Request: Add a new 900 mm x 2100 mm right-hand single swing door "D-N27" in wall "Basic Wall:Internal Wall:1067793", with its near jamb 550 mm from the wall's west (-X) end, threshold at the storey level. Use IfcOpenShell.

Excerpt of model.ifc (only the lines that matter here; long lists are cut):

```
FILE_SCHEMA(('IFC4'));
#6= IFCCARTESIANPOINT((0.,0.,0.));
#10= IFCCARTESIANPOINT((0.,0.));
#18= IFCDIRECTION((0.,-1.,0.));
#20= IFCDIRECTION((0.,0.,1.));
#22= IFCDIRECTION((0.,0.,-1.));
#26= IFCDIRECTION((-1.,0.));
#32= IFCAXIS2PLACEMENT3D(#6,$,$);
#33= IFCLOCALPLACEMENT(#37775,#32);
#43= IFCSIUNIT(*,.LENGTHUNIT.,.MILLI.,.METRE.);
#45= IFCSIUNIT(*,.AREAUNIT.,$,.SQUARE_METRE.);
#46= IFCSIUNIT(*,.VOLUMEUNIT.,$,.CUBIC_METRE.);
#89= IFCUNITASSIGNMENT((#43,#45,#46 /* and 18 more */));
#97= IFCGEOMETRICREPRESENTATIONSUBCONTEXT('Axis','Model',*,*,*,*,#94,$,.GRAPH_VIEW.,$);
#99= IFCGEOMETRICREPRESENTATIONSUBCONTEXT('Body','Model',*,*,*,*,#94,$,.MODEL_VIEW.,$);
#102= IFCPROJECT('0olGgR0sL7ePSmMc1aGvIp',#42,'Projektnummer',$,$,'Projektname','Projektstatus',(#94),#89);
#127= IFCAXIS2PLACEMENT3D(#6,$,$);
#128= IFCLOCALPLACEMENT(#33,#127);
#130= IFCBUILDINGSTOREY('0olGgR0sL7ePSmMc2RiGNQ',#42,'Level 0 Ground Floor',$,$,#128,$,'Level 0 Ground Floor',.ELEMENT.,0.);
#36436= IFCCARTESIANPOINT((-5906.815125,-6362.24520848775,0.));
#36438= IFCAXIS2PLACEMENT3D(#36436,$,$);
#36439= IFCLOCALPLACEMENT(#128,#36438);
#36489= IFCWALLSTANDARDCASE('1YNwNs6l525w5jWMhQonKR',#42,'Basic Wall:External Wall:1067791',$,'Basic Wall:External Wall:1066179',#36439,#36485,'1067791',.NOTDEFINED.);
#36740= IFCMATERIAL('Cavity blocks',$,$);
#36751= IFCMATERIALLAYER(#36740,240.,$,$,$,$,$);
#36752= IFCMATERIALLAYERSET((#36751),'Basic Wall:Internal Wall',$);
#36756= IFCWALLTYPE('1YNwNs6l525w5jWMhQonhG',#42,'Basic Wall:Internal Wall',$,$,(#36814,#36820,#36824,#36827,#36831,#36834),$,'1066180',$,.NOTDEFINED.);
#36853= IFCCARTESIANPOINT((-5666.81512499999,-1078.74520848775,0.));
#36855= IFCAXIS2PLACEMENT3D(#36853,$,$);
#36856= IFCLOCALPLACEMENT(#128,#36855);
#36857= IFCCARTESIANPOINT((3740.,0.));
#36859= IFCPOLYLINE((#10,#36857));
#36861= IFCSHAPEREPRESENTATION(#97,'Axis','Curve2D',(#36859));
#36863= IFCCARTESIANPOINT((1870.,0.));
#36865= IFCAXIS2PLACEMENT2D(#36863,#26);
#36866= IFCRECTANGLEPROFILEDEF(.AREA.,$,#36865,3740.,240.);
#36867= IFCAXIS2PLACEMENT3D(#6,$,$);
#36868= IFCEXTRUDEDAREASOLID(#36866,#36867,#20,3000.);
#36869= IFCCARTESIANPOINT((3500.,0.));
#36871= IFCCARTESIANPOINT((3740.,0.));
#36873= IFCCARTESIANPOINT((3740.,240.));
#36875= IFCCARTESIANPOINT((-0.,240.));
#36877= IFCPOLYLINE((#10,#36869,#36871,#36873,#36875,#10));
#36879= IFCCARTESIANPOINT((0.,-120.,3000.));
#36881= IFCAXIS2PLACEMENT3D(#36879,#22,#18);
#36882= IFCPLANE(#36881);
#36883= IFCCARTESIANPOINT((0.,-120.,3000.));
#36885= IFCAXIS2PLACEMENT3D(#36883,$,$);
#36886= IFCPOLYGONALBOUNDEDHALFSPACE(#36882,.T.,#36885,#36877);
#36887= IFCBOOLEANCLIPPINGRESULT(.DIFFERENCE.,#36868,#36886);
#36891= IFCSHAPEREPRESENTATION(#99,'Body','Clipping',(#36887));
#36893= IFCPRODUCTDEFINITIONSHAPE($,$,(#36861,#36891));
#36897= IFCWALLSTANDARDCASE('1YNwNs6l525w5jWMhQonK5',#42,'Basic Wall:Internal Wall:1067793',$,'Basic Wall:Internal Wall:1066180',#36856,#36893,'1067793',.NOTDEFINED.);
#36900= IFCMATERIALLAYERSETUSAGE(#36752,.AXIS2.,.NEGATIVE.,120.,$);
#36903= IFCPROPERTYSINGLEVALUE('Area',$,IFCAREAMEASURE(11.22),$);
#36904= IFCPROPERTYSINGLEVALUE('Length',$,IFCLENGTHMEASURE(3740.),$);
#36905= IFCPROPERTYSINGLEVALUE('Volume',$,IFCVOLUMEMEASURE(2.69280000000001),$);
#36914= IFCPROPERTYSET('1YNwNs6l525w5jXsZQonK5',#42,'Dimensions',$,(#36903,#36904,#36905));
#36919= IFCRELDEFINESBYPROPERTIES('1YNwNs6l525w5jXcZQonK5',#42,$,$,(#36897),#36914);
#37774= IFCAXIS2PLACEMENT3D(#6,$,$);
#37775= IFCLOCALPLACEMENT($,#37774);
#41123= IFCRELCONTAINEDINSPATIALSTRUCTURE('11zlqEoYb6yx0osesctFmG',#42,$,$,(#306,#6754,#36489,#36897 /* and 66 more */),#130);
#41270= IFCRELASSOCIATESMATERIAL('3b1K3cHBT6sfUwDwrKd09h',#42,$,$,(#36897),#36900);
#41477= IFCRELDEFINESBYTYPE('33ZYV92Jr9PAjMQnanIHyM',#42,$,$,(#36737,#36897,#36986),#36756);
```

```python
import numpy as np
import ifcopenshell
import ifcopenshell.api.feature
import ifcopenshell.api.geometry
import ifcopenshell.api.pset
import ifcopenshell.api.root
import ifcopenshell.api.spatial
import ifcopenshell.geom
import ifcopenshell.util.element
import ifcopenshell.util.placement
import ifcopenshell.util.representation
import ifcopenshell.util.shape
import ifcopenshell.util.unit

model = ifcopenshell.open("model.ifc")
unit_scale = ifcopenshell.util.unit.calculate_unit_scale(model)
area_scale = ifcopenshell.util.unit.calculate_unit_scale(model, "AREAUNIT")
volume_scale = ifcopenshell.util.unit.calculate_unit_scale(model, "VOLUMEUNIT")
settings = ifcopenshell.geom.settings()


def volume(element):
    """Net volume in cubic metres, openings subtracted."""
    shape = ifcopenshell.geom.create_shape(settings, element)
    return ifcopenshell.util.shape.get_volume(shape.geometry)


wall = model.by_guid("1YNwNs6l525w5jWMhQonK5")
storey = ifcopenshell.util.element.get_container(wall, ifc_class="IfcBuildingStorey")
context = ifcopenshell.util.representation.get_context(model, "Model", "Body", "MODEL_VIEW")
before = volume(wall)

width, height, from_end, sill = 0.9, 2.1, 0.55, 0.0  # metres

# The wall runs along its own X axis, and the end named is its -X end.
wall_shape = ifcopenshell.geom.create_shape(settings, wall)
x, y, z = ifcopenshell.util.shape.get_vertices(wall_shape.geometry).T
start = x.min() + from_end
face, thickness = float(y.min()), float(y.max() - y.min())
wall_matrix = ifcopenshell.util.placement.get_local_placement(wall.ObjectPlacement)
level = ifcopenshell.util.placement.get_local_placement(storey.ObjectPlacement)[2, 3]


def in_wall(x, y):
    """Placement at x, y metres in the wall's axes, at sill height."""
    matrix = wall_matrix.copy()
    matrix[:, 3] = wall_matrix @ np.array([x / unit_scale, y / unit_scale, 0.0, 1.0])
    matrix[2, 3] = level + sill / unit_scale
    return matrix


# Opening: a box that overshoots both wall faces by 50 mm.
opening = ifcopenshell.api.root.create_entity(model, ifc_class="IfcOpeningElement", predefined_type="OPENING")
box = ifcopenshell.api.geometry.add_wall_representation(
    model, context=context, length=width, height=height, thickness=thickness + 0.1
)
ifcopenshell.api.geometry.assign_representation(model, product=opening, representation=box)
ifcopenshell.api.geometry.edit_object_placement(model, product=opening, matrix=in_wall(start, face - 0.05), is_si=False)
ifcopenshell.api.feature.add_feature(model, feature=opening, element=wall)

door = ifcopenshell.api.root.create_entity(model, ifc_class="IfcDoor", name="D-N27", predefined_type="DOOR")
door.OverallWidth, door.OverallHeight = width / unit_scale, height / unit_scale
door.OperationType = "SINGLE_SWING_RIGHT"
body = ifcopenshell.api.geometry.add_door_representation(
    model,
    context=context,
    overall_width=door.OverallWidth,
    overall_height=door.OverallHeight,
    operation_type="SINGLE_SWING_RIGHT",
    lining_properties={"LiningDepth": thickness / unit_scale, "ThresholdDepth": thickness / unit_scale},
)
ifcopenshell.api.geometry.assign_representation(model, product=door, representation=body)
ifcopenshell.api.spatial.assign_container(model, products=[door], relating_structure=storey)
ifcopenshell.api.feature.add_filling(model, opening=opening, element=door)

# The lining spans the wall, so the door starts at the wall face.
ifcopenshell.api.geometry.edit_object_placement(model, product=door, matrix=in_wall(start, face), is_si=False)

after = volume(wall)

# Update the wall's stored quantities.
pset = model.by_id(ifcopenshell.util.element.get_pset(wall, "Dimensions", should_inherit=False)["id"])
ifcopenshell.api.pset.edit_pset(model, pset=pset, properties={
    "Area": model.create_entity("IfcAreaMeasure", after / thickness / area_scale),
    "Volume": model.create_entity("IfcVolumeMeasure", after / volume_scale),
})

print(f"wall volume {before:.3f} -> {after:.3f} m3")

model.write("model_updated.ifc")
```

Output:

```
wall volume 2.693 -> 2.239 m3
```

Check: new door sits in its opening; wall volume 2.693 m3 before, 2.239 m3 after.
